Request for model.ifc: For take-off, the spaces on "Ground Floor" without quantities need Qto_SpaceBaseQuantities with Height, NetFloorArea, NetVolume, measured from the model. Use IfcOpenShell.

First a look at what the model holds.

```python
import ifcopenshell
import ifcopenshell.util.element
import ifcopenshell.util.unit

model = ifcopenshell.open("model.ifc")
print(model.schema)
for unit_type in ("LENGTHUNIT", "AREAUNIT", "VOLUMEUNIT"):
    print(unit_type, ifcopenshell.util.unit.calculate_unit_scale(model, unit_type))
storey = next(s for s in model.by_type("IfcBuildingStorey") if s.Name == "Ground Floor")
spaces = [e for e in ifcopenshell.util.element.get_decomposition(storey) if e.is_a("IfcSpace")]
for e in sorted(spaces, key=lambda e: e.id()):
    print(e.id(), e.is_a(), e.Name, list(ifcopenshell.util.element.get_psets(e, qtos_only=True)), sep=" | ")
```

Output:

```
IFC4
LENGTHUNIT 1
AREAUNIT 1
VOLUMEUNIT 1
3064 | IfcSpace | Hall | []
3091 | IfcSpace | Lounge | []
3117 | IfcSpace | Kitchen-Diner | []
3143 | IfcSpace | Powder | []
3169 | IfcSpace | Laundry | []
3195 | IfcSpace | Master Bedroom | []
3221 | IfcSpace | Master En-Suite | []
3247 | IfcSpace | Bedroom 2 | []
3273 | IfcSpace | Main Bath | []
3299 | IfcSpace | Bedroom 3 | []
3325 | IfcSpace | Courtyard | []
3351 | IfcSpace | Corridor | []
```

```python
import ifcopenshell
import ifcopenshell.api.pset
import ifcopenshell.geom
import ifcopenshell.util.element
import ifcopenshell.util.shape
import ifcopenshell.util.unit

model = ifcopenshell.open("model.ifc")
unit_scale = ifcopenshell.util.unit.calculate_unit_scale(model)
area_scale = ifcopenshell.util.unit.calculate_unit_scale(model, "AREAUNIT")
volume_scale = ifcopenshell.util.unit.calculate_unit_scale(model, "VOLUMEUNIT")
settings = ifcopenshell.geom.settings()

storey = next(s for s in model.by_type("IfcBuildingStorey") if s.Name == "Ground Floor")
spaces = [e for e in ifcopenshell.util.element.get_decomposition(storey) if e.is_a("IfcSpace")]

for e in sorted(spaces, key=lambda e: e.id()):
    if ifcopenshell.util.element.get_psets(e, qtos_only=True, should_inherit=False):
        continue
    # Geometry comes back in metres, in the element's own axes.
    shape = ifcopenshell.geom.create_shape(settings, e)
    values = {
        "Height": ifcopenshell.util.shape.get_z(shape.geometry) / unit_scale,
        "NetFloorArea": ifcopenshell.util.shape.get_footprint_area(shape.geometry) / area_scale,
        "NetVolume": ifcopenshell.util.shape.get_volume(shape.geometry) / volume_scale,
    }
    qto = ifcopenshell.api.pset.add_qto(model, product=e, name="Qto_SpaceBaseQuantities")
    ifcopenshell.api.pset.edit_qto(model, qto=qto, properties=values)
    print(e.id(), {k: round(v, 3) for k, v in values.items()})

model.write("model_edited.ifc")
```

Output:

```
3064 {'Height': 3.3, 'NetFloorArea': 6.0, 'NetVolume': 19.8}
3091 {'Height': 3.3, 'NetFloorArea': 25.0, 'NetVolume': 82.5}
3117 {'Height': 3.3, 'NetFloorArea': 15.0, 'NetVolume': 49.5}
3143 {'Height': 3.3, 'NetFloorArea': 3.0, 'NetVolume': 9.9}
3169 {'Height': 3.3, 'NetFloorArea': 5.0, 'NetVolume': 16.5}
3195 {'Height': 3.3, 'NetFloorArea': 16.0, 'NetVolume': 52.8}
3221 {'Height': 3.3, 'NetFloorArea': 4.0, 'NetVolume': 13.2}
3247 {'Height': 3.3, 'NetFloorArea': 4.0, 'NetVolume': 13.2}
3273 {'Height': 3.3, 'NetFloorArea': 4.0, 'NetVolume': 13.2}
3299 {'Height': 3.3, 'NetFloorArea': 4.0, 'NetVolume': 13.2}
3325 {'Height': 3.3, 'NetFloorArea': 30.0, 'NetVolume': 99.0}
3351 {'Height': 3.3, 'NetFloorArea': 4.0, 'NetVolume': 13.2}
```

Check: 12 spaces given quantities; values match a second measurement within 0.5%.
